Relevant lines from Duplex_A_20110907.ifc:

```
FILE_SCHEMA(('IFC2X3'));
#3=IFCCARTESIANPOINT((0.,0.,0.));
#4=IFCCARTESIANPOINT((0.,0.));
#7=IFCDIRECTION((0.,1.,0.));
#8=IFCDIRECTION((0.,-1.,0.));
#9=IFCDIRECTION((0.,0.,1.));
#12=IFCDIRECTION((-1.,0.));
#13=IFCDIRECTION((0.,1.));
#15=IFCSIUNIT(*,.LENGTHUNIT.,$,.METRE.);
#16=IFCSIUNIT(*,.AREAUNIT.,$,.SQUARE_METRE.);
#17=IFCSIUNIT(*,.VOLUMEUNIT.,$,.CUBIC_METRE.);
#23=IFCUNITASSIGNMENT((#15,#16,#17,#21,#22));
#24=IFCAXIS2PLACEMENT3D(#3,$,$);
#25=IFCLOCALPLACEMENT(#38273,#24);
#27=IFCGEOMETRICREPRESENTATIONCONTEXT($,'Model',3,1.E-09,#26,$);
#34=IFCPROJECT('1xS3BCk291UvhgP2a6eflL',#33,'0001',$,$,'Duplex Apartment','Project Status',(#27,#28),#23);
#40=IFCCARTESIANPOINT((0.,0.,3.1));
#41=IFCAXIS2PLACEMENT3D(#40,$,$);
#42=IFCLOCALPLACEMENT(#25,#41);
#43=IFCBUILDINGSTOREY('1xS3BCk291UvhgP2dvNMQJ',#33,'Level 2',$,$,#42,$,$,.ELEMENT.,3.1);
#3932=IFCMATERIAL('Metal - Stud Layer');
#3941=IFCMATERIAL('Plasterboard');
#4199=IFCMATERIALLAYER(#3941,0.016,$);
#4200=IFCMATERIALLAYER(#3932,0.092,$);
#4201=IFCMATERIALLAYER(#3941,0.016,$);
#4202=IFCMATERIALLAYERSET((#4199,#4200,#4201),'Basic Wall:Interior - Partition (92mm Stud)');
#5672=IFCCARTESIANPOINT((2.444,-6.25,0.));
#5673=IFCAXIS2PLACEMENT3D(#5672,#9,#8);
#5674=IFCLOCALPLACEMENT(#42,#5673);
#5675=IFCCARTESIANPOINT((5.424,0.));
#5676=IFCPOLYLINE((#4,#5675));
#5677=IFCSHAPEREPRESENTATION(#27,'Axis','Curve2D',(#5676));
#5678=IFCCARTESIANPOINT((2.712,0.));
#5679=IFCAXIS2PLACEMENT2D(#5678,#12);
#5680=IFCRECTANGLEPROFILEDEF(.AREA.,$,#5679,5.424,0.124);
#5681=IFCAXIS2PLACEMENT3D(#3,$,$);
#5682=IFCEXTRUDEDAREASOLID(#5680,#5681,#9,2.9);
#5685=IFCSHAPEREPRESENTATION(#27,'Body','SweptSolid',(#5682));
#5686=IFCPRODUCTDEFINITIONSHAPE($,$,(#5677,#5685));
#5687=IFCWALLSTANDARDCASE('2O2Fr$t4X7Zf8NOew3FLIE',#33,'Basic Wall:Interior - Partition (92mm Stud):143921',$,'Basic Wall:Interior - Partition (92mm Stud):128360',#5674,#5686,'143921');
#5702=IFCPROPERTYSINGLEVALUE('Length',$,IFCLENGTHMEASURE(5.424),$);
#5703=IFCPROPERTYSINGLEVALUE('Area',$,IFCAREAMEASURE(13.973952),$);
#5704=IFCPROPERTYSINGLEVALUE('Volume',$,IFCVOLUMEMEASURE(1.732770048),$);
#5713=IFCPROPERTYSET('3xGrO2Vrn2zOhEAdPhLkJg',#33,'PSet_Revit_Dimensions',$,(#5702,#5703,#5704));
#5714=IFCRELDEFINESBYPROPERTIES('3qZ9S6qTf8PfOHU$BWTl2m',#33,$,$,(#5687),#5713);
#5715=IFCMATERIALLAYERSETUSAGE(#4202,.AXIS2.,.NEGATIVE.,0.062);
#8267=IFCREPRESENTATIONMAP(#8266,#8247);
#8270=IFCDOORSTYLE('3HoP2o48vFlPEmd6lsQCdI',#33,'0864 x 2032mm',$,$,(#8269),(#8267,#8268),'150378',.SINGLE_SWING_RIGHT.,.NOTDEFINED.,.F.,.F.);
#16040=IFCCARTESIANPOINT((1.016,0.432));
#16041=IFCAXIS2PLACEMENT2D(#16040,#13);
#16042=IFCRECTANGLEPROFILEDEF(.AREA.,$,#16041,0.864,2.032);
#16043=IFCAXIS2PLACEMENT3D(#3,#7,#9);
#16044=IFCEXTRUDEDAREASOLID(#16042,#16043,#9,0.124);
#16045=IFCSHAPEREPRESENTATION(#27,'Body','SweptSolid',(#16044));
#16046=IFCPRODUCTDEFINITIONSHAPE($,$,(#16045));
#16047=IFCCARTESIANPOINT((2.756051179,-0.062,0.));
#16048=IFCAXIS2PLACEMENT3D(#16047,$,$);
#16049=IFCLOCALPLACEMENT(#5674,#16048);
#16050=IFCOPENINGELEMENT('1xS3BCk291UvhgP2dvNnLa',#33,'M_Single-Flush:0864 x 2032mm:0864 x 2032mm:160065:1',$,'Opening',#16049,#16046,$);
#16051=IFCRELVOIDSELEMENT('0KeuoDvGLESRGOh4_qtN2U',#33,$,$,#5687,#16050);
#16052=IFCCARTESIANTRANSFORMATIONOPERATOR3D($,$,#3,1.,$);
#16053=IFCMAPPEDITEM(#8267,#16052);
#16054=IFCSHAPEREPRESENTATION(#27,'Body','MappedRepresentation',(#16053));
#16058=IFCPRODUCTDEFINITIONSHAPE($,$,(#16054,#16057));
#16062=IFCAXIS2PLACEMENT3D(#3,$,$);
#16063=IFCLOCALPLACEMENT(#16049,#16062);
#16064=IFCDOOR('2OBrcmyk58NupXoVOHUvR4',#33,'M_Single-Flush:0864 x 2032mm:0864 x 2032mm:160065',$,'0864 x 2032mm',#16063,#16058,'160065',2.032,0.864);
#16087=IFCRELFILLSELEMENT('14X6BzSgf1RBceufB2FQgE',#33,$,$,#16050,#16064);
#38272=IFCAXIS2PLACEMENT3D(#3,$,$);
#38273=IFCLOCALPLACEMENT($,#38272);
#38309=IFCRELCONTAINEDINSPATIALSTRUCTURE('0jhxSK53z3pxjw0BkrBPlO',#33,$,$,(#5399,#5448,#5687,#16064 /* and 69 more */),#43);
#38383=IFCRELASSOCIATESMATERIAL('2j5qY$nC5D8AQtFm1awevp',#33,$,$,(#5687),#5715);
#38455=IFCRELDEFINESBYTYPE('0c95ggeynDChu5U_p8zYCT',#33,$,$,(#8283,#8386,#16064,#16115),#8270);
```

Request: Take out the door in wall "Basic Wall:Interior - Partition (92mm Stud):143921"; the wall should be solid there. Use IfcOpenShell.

```python
import ifcopenshell
import ifcopenshell.api.feature
import ifcopenshell.api.pset
import ifcopenshell.api.root
import ifcopenshell.geom
import ifcopenshell.util.element
import ifcopenshell.util.shape
import ifcopenshell.util.unit

model = ifcopenshell.open("Duplex_A_20110907.ifc")
area_scale = ifcopenshell.util.unit.calculate_unit_scale(model, "AREAUNIT")
volume_scale = ifcopenshell.util.unit.calculate_unit_scale(model, "VOLUMEUNIT")
settings = ifcopenshell.geom.settings()


def volume(element):
    """Net volume in cubic metres, openings subtracted."""
    shape = ifcopenshell.geom.create_shape(settings, element)
    return ifcopenshell.util.shape.get_volume(shape.geometry)


door = model.by_guid("2OBrcmyk58NupXoVOHUvR4")
opening = door.FillsVoids[0].RelatingOpeningElement
wall = opening.VoidsElements[0].RelatingBuildingElement
before = volume(wall)

ifcopenshell.api.root.remove_product(model, product=door)
ifcopenshell.api.feature.remove_feature(model, feature=opening)

after = volume(wall)
thickness = 0.124  # wall thickness in metres

# Update the wall's stored quantities.
pset = model.by_id(ifcopenshell.util.element.get_pset(wall, "PSet_Revit_Dimensions", should_inherit=False)["id"])
ifcopenshell.api.pset.edit_pset(model, pset=pset, properties={
    "Area": model.create_entity("IfcAreaMeasure", after / thickness / area_scale),
    "Volume": model.create_entity("IfcVolumeMeasure", after / volume_scale),
})

print(f"wall volume {before:.3f} -> {after:.3f} m3")

model.write("Duplex_A_20110907_rev.ifc")
```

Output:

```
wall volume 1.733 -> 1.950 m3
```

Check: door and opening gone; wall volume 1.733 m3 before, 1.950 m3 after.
